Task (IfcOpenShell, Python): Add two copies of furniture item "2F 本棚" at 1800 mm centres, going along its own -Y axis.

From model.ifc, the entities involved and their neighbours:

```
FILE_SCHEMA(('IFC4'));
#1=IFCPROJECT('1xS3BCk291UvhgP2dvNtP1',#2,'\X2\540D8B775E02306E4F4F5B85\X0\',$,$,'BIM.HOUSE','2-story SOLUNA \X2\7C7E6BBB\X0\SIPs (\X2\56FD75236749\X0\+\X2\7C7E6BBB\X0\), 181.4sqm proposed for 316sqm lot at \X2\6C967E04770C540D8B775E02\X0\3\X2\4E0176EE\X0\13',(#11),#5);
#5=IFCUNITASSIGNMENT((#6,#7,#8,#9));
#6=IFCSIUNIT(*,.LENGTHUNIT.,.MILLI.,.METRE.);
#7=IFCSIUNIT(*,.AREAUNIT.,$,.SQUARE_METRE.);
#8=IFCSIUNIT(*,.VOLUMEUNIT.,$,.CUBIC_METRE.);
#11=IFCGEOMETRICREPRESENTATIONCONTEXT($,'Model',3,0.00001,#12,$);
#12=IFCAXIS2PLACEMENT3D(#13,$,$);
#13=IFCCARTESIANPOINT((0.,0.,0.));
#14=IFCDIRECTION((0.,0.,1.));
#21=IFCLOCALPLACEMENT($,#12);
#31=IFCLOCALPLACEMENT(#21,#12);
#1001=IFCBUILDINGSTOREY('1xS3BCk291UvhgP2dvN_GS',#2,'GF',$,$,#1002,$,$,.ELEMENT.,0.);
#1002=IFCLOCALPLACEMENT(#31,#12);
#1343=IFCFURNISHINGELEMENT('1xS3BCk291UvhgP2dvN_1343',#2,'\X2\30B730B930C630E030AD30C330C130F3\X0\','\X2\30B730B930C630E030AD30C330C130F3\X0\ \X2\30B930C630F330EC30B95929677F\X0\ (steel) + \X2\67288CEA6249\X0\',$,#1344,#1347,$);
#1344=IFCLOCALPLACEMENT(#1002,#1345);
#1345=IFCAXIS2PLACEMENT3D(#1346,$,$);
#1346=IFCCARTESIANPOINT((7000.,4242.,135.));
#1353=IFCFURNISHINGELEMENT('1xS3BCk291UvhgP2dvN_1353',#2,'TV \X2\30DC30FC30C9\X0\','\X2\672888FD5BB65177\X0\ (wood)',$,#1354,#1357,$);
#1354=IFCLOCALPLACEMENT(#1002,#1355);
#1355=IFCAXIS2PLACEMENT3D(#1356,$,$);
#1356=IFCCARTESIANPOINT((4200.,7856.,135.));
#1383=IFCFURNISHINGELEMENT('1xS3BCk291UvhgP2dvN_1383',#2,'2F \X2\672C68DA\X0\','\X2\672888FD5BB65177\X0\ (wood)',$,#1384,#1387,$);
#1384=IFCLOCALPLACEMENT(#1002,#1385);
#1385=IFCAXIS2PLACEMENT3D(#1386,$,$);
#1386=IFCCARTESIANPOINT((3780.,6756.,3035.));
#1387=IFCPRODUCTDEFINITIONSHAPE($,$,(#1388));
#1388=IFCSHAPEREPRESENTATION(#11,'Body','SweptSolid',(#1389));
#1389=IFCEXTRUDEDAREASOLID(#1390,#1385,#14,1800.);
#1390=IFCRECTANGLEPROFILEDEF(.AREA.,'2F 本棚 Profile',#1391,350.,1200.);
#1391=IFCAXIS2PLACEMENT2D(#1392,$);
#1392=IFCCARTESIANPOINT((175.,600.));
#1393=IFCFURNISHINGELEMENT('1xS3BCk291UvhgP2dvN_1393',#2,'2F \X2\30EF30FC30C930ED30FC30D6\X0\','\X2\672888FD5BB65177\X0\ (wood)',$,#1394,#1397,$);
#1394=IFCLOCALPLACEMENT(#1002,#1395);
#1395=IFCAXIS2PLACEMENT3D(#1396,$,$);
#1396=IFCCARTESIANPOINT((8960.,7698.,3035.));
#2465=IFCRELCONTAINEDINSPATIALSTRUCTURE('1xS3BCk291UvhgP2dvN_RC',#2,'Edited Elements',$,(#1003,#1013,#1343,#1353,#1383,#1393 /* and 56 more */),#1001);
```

```python
import ifcopenshell
import ifcopenshell.api.geometry
import ifcopenshell.api.root
import ifcopenshell.util.element
import ifcopenshell.util.placement
import ifcopenshell.util.unit

model = ifcopenshell.open("model.ifc")
unit_scale = ifcopenshell.util.unit.calculate_unit_scale(model)


def reuse_history(source, copy):
    """copy_class also copies each property set's owner history, people and application; keep the originals."""
    for rel in copy.IsDefinedBy:
        if rel.is_a("IfcRelDefinesByProperties") and (history := rel.RelatingPropertyDefinition.OwnerHistory):
            rel.RelatingPropertyDefinition.OwnerHistory = source.OwnerHistory
            ifcopenshell.util.element.remove_deep2(model, history)


source = model.by_guid("1xS3BCk291UvhgP2dvN_1383")
base = ifcopenshell.util.placement.get_local_placement(source.ObjectPlacement)
step = -base[:3, 1] * 1.8 / unit_scale

for i in range(1, 3):
    copy = ifcopenshell.api.root.copy_class(model, product=source)
    copy.Representation = ifcopenshell.util.element.copy_deep(
        model, source.Representation, exclude=["IfcGeometricRepresentationContext", "IfcRepresentationMap"]
    )
    reuse_history(source, copy)
    matrix = base.copy()
    matrix[:3, 3] += i * step
    print("added at", matrix[:3, 3].round(3) + 0.0)
    ifcopenshell.api.geometry.edit_object_placement(model, product=copy, matrix=matrix, is_si=False)

model.write("model_rev.ifc")
```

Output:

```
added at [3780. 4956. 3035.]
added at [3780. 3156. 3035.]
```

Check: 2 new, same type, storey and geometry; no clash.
